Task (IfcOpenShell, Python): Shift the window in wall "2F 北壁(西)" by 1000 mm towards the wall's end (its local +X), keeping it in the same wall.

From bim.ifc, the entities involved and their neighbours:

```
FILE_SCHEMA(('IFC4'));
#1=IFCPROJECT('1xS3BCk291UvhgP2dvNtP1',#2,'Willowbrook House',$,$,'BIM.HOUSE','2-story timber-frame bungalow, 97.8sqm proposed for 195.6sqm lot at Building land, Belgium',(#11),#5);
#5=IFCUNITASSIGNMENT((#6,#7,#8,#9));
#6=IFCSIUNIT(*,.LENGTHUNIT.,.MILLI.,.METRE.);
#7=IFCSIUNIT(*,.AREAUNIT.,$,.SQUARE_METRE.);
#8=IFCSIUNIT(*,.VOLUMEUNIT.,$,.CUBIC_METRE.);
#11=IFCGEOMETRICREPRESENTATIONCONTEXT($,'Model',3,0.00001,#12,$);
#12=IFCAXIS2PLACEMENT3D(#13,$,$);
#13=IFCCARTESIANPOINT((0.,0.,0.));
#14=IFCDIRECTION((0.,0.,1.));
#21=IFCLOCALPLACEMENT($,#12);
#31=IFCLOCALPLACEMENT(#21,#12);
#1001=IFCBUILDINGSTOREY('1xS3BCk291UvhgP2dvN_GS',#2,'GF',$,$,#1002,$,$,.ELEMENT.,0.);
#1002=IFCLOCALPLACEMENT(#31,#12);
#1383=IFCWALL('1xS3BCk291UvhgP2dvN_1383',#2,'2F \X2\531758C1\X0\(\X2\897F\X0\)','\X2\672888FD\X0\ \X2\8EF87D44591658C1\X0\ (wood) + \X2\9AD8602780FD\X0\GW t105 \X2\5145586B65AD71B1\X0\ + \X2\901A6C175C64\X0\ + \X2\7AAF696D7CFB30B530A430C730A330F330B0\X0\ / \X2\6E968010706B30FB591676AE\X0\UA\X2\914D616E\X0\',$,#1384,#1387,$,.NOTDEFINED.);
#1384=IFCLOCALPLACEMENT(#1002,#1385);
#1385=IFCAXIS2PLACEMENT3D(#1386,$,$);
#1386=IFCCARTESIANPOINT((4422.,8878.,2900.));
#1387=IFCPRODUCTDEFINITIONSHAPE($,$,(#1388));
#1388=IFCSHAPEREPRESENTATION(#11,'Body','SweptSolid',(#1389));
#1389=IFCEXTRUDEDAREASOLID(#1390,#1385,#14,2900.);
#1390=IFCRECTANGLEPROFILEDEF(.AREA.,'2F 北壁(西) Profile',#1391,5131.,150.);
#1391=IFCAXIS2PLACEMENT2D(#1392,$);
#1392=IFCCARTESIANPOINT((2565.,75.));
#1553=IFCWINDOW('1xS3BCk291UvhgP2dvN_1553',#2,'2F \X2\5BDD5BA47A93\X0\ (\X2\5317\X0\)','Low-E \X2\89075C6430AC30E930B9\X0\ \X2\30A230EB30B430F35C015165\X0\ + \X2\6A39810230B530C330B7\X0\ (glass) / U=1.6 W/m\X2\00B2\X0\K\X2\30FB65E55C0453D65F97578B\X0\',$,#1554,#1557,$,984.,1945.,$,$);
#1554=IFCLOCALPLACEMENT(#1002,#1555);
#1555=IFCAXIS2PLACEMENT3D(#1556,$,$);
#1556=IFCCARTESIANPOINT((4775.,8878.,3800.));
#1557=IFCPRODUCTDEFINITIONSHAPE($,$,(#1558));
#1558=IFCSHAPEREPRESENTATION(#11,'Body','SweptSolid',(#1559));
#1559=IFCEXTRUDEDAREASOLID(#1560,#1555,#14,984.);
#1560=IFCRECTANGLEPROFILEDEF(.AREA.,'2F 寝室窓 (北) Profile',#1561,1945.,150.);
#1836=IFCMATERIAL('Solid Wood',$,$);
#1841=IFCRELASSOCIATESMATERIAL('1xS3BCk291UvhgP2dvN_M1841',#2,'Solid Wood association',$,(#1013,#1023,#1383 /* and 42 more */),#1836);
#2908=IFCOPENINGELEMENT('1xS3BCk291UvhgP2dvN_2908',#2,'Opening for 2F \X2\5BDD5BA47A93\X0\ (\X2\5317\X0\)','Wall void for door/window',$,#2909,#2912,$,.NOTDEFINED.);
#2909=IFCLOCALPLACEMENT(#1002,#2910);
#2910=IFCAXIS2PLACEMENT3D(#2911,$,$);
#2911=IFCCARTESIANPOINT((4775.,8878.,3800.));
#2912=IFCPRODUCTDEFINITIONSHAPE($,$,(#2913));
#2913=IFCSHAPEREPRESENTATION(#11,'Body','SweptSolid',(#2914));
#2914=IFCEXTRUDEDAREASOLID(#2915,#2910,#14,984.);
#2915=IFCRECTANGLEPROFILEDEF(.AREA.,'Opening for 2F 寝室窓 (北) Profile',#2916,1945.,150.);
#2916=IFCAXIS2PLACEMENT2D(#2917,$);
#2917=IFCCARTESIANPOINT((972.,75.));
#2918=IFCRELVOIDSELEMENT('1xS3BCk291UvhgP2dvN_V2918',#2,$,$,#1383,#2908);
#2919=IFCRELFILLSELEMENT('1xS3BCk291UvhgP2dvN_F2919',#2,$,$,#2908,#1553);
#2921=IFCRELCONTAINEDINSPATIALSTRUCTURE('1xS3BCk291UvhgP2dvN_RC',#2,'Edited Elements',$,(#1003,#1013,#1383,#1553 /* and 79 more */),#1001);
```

```python
import ifcopenshell
import ifcopenshell.api.geometry
import ifcopenshell.util.placement
import ifcopenshell.util.unit

model = ifcopenshell.open("bim.ifc")
unit_scale = ifcopenshell.util.unit.calculate_unit_scale(model)

window = model.by_guid("1xS3BCk291UvhgP2dvN_1553")
opening = window.FillsVoids[0].RelatingOpeningElement
wall = opening.VoidsElements[0].RelatingBuildingElement

wall_matrix = ifcopenshell.util.placement.get_local_placement(wall.ObjectPlacement)
shift = wall_matrix[:3, 0] * 1 / unit_scale
before = ifcopenshell.util.placement.get_local_placement(window.ObjectPlacement)[:3, 3].copy()

# The window is not placed relative to its opening, so move both.
for product in (opening, window):
    matrix = ifcopenshell.util.placement.get_local_placement(product.ObjectPlacement)
    matrix[:3, 3] += shift
    ifcopenshell.api.geometry.edit_object_placement(model, product=product, matrix=matrix, is_si=False)

after = ifcopenshell.util.placement.get_local_placement(window.ObjectPlacement)[:3, 3]
print("window moved by", (after - before).round(3) + 0.0)

model.write("bim_updated.ifc")
```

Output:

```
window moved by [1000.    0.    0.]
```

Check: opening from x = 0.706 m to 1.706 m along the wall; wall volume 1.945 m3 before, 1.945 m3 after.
